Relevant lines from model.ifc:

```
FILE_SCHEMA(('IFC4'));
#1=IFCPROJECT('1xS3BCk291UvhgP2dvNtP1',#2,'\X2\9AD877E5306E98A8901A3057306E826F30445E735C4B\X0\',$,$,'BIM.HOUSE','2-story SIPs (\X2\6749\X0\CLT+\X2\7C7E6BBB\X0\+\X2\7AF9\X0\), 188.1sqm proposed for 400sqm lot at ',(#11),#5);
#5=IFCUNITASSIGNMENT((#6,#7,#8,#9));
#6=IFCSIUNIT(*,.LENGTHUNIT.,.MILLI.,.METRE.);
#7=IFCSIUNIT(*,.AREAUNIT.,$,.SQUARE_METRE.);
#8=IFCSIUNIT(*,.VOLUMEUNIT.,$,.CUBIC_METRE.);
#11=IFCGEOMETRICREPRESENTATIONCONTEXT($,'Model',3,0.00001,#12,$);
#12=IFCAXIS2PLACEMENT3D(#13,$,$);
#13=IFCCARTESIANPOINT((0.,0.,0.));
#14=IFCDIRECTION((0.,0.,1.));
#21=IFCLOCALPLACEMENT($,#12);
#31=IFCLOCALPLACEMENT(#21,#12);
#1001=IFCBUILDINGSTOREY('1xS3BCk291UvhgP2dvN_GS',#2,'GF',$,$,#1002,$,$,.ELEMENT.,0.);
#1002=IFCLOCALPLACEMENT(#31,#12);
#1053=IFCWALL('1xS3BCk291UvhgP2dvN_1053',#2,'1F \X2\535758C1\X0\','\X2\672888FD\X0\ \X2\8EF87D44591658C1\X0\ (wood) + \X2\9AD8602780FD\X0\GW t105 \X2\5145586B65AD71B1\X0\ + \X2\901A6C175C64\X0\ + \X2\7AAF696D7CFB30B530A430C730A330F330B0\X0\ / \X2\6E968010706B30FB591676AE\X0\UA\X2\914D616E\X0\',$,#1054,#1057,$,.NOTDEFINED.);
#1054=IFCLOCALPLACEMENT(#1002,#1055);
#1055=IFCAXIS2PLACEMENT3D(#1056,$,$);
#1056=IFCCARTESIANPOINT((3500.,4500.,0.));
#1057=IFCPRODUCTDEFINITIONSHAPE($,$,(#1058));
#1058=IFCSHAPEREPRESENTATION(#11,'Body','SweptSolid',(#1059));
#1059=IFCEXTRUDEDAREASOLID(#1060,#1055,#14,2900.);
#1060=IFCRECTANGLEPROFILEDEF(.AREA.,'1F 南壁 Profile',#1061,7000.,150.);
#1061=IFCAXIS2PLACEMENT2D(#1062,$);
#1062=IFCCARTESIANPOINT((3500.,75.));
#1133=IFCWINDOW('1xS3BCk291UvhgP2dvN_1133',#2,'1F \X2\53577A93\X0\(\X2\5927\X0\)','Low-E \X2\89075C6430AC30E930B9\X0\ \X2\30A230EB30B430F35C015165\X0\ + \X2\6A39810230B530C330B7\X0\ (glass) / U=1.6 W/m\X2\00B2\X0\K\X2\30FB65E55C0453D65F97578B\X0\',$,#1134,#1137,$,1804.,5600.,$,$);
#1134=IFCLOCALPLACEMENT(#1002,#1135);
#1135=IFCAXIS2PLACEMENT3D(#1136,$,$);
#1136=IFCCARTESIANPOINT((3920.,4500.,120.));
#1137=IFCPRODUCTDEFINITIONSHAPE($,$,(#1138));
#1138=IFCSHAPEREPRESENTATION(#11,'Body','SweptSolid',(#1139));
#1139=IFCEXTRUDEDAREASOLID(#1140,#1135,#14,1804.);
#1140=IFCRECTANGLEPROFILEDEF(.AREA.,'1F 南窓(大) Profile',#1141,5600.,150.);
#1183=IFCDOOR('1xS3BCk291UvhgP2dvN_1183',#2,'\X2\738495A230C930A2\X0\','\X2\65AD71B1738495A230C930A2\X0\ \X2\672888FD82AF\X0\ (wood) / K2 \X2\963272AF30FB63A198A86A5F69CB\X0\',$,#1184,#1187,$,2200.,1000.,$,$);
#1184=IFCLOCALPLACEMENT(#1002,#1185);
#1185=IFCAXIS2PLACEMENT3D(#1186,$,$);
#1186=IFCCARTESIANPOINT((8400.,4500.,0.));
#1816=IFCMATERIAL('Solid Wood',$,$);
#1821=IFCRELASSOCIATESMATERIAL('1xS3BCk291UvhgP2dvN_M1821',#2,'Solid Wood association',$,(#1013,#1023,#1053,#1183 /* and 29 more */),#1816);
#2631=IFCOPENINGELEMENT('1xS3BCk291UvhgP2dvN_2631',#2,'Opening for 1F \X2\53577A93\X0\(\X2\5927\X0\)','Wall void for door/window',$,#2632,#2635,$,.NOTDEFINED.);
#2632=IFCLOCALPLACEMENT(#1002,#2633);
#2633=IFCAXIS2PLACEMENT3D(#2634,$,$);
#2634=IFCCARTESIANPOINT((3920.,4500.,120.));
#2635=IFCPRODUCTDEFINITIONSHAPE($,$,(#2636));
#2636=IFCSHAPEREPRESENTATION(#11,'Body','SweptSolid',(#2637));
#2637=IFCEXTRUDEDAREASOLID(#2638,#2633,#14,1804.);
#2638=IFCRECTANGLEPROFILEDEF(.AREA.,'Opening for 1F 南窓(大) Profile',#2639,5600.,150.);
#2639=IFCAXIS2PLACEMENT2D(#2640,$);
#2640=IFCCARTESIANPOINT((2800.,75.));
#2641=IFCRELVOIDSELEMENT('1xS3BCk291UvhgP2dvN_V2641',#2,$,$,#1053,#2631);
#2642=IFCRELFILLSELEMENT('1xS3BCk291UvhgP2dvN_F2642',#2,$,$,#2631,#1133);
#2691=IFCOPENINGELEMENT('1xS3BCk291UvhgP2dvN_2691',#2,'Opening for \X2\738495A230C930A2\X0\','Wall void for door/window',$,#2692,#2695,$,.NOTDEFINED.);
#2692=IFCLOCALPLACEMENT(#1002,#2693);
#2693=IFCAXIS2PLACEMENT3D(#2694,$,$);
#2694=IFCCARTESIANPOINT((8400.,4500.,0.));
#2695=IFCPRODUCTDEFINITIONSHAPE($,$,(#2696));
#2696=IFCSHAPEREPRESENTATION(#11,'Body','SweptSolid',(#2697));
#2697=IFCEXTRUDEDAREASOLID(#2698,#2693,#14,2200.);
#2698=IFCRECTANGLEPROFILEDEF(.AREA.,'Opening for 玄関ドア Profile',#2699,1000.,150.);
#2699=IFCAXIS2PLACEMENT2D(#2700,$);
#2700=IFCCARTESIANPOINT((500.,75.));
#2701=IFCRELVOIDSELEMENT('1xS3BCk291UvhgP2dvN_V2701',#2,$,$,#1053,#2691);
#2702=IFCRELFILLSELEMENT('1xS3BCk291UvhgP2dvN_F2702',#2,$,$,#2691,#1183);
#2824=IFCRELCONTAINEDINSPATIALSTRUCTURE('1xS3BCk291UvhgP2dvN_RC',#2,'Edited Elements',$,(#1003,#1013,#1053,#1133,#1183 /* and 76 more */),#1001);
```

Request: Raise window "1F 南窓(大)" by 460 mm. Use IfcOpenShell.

```python
import numpy as np
import ifcopenshell
import ifcopenshell.api.geometry
import ifcopenshell.util.placement
import ifcopenshell.util.unit

model = ifcopenshell.open("model.ifc")
unit_scale = ifcopenshell.util.unit.calculate_unit_scale(model)

window = model.by_guid("1xS3BCk291UvhgP2dvN_1133")
opening = window.FillsVoids[0].RelatingOpeningElement
dz = 0.46 / unit_scale

shift = np.array([0.0, 0.0, dz])
# The window is not placed relative to its opening, so move both.
for product in (opening, window):
    matrix = ifcopenshell.util.placement.get_local_placement(product.ObjectPlacement)
    matrix[:3, 3] += shift
    ifcopenshell.api.geometry.edit_object_placement(model, product=product, matrix=matrix, is_si=False)

print(f"moved by {dz * unit_scale:+.3f} m")

model.write("model_rev.ifc")
```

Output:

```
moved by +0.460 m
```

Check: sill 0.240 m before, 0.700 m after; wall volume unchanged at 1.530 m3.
